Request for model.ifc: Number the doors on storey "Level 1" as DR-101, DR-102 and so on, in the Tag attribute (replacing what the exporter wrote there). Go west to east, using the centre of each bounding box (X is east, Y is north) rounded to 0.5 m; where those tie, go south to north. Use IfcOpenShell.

First a look at what the model holds.

```python
import ifcopenshell
import ifcopenshell.util.element
import ifcopenshell.util.placement

model = ifcopenshell.open("model.ifc")
print(model.schema)
storey = next(s for s in model.by_type("IfcBuildingStorey") if s.Name == "Level 1")
doors = [e for e in ifcopenshell.util.element.get_decomposition(storey) if e.is_a("IfcDoor")]
for e in sorted(doors, key=lambda e: e.id()):
    origin = ifcopenshell.util.placement.get_local_placement(e.ObjectPlacement)[:3, 3]
    print(e.id(), e.Tag, e.Name, origin.round(2) + 0.0, sep=" | ")
```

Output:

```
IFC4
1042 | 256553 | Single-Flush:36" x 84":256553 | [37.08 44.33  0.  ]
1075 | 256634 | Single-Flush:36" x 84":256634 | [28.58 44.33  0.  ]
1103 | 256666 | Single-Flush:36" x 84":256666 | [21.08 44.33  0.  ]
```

```python
import ifcopenshell
import ifcopenshell.geom
import ifcopenshell.util.element
import ifcopenshell.util.shape

model = ifcopenshell.open("model.ifc")
settings = ifcopenshell.geom.settings()
settings.set("use-world-coords", True)


def centre(element):
    shape = ifcopenshell.geom.create_shape(settings, element)
    return ifcopenshell.util.shape.get_bbox_centroid(shape.geometry)


storey = next(s for s in model.by_type("IfcBuildingStorey") if s.Name == "Level 1")
doors = [e for e in ifcopenshell.util.element.get_decomposition(storey) if e.is_a("IfcDoor")]

# Insertion points can sit at a corner or the storey origin, so sort by the geometry (in metres).
centres = {e: centre(e) for e in doors}
doors.sort(key=lambda e: (round(centres[e][0] / 0.5), centres[e][1]))

for i, e in enumerate(doors, start=1):
    number = f"DR-1{i:02d}"
    e.Tag = number
    print(e.id(), number)

model.write("model_rev.ifc")
```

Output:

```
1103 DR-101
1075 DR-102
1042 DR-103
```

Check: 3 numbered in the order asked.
